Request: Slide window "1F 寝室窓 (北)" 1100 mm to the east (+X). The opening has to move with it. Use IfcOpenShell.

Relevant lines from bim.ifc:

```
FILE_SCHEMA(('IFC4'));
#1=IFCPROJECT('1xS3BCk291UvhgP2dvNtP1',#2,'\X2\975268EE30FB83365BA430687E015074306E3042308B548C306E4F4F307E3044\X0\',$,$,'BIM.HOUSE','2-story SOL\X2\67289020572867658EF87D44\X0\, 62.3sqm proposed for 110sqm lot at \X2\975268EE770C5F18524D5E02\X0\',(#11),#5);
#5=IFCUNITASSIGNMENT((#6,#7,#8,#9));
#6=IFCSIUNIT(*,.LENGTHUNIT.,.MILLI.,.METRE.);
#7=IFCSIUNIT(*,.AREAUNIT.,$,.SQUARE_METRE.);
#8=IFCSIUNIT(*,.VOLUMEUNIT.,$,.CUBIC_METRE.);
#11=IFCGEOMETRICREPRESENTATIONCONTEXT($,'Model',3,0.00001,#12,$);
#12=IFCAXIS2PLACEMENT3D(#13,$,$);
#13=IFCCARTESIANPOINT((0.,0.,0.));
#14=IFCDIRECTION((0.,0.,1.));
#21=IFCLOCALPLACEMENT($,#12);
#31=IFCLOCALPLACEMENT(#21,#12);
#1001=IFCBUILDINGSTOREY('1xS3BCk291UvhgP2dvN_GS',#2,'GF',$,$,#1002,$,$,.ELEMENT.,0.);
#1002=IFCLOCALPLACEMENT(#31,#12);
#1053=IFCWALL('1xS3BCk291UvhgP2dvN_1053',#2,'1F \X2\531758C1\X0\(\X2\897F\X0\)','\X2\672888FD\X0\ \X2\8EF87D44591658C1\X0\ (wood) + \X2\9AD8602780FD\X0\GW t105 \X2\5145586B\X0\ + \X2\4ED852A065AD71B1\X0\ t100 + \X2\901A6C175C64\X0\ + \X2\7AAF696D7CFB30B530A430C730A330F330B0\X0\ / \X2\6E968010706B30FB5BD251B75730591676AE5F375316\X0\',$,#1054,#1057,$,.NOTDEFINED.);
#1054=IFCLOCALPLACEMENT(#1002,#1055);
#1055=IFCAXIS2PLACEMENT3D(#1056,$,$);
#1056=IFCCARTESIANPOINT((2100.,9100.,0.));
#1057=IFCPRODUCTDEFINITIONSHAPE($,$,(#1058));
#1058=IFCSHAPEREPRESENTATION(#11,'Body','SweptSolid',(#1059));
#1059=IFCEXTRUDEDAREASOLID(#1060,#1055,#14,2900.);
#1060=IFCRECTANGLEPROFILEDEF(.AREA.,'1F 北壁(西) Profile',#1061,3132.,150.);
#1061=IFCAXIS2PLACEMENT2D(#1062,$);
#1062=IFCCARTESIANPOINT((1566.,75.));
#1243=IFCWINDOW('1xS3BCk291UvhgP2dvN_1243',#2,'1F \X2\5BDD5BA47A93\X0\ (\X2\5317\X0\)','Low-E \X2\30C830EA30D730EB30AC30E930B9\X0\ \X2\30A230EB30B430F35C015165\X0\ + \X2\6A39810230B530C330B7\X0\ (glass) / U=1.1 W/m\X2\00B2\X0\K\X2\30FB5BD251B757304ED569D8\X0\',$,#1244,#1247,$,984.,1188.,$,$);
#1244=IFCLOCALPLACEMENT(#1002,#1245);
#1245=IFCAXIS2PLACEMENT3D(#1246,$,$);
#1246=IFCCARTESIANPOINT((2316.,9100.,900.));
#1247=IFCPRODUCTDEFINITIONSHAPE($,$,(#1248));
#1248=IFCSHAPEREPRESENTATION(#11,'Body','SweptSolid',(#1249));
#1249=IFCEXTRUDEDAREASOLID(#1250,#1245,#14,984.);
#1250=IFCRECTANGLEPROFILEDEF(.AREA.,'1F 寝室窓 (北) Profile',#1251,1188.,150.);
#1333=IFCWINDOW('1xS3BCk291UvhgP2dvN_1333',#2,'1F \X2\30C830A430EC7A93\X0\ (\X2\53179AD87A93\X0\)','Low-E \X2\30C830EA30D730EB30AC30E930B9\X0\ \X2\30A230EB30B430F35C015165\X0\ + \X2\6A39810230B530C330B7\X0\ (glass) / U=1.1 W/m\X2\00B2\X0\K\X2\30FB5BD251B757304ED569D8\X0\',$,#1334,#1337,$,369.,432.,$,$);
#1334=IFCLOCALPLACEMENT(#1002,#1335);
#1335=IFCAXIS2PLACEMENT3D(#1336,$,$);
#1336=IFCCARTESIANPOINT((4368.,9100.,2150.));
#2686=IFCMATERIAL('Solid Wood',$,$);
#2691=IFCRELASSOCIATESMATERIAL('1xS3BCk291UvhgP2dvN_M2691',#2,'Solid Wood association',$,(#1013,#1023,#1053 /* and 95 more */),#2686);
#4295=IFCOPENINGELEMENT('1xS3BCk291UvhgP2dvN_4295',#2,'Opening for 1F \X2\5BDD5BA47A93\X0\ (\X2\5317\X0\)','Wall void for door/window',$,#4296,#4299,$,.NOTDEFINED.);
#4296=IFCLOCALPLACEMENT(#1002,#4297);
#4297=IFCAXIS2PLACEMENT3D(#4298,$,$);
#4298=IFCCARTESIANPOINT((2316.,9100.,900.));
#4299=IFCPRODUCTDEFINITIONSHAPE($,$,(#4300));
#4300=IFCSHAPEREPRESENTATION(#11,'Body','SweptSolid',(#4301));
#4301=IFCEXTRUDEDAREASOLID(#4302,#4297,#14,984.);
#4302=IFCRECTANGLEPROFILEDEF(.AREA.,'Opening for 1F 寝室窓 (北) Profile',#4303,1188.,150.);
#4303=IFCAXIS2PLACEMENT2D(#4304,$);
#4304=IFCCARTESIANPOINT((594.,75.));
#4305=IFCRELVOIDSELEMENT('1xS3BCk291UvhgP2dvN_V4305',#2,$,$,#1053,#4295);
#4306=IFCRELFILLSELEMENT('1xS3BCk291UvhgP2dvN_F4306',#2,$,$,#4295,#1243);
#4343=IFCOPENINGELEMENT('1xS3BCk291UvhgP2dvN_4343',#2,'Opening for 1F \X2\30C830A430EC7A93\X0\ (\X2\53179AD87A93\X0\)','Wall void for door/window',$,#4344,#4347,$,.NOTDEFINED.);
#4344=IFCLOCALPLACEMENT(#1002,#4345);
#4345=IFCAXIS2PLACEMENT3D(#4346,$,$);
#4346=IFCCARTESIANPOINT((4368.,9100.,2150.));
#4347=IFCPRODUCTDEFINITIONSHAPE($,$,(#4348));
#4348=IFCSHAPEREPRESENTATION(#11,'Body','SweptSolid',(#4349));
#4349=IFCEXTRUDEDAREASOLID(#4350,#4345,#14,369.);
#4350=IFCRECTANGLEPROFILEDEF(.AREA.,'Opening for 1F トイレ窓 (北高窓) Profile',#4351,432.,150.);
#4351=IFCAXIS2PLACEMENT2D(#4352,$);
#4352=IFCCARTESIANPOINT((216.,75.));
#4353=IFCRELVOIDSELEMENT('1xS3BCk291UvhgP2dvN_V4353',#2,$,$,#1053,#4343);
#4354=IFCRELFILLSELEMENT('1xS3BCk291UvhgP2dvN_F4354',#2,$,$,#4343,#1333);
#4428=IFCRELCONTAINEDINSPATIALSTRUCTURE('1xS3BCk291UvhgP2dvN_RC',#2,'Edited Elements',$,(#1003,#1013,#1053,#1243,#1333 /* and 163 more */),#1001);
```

```python
import ifcopenshell
import ifcopenshell.api.geometry
import ifcopenshell.util.placement

model = ifcopenshell.open("bim.ifc")

window = model.by_guid("1xS3BCk291UvhgP2dvN_1243")
opening = window.FillsVoids[0].RelatingOpeningElement
wall = opening.VoidsElements[0].RelatingBuildingElement

wall_matrix = ifcopenshell.util.placement.get_local_placement(wall.ObjectPlacement)
shift = wall_matrix[:3, 0] * 1100.0
before = ifcopenshell.util.placement.get_local_placement(window.ObjectPlacement)[:3, 3].copy()

# The window is not placed relative to its opening, so move both.
for product in (opening, window):
    matrix = ifcopenshell.util.placement.get_local_placement(product.ObjectPlacement)
    matrix[:3, 3] += shift
    ifcopenshell.api.geometry.edit_object_placement(model, product=product, matrix=matrix, is_si=False)

after = ifcopenshell.util.placement.get_local_placement(window.ObjectPlacement)[:3, 3]
print("window moved by", (after - before).round(3) + 0.0)

model.write("bim_edited.ifc")
```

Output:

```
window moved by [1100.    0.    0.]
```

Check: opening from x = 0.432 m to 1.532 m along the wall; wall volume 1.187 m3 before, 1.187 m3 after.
